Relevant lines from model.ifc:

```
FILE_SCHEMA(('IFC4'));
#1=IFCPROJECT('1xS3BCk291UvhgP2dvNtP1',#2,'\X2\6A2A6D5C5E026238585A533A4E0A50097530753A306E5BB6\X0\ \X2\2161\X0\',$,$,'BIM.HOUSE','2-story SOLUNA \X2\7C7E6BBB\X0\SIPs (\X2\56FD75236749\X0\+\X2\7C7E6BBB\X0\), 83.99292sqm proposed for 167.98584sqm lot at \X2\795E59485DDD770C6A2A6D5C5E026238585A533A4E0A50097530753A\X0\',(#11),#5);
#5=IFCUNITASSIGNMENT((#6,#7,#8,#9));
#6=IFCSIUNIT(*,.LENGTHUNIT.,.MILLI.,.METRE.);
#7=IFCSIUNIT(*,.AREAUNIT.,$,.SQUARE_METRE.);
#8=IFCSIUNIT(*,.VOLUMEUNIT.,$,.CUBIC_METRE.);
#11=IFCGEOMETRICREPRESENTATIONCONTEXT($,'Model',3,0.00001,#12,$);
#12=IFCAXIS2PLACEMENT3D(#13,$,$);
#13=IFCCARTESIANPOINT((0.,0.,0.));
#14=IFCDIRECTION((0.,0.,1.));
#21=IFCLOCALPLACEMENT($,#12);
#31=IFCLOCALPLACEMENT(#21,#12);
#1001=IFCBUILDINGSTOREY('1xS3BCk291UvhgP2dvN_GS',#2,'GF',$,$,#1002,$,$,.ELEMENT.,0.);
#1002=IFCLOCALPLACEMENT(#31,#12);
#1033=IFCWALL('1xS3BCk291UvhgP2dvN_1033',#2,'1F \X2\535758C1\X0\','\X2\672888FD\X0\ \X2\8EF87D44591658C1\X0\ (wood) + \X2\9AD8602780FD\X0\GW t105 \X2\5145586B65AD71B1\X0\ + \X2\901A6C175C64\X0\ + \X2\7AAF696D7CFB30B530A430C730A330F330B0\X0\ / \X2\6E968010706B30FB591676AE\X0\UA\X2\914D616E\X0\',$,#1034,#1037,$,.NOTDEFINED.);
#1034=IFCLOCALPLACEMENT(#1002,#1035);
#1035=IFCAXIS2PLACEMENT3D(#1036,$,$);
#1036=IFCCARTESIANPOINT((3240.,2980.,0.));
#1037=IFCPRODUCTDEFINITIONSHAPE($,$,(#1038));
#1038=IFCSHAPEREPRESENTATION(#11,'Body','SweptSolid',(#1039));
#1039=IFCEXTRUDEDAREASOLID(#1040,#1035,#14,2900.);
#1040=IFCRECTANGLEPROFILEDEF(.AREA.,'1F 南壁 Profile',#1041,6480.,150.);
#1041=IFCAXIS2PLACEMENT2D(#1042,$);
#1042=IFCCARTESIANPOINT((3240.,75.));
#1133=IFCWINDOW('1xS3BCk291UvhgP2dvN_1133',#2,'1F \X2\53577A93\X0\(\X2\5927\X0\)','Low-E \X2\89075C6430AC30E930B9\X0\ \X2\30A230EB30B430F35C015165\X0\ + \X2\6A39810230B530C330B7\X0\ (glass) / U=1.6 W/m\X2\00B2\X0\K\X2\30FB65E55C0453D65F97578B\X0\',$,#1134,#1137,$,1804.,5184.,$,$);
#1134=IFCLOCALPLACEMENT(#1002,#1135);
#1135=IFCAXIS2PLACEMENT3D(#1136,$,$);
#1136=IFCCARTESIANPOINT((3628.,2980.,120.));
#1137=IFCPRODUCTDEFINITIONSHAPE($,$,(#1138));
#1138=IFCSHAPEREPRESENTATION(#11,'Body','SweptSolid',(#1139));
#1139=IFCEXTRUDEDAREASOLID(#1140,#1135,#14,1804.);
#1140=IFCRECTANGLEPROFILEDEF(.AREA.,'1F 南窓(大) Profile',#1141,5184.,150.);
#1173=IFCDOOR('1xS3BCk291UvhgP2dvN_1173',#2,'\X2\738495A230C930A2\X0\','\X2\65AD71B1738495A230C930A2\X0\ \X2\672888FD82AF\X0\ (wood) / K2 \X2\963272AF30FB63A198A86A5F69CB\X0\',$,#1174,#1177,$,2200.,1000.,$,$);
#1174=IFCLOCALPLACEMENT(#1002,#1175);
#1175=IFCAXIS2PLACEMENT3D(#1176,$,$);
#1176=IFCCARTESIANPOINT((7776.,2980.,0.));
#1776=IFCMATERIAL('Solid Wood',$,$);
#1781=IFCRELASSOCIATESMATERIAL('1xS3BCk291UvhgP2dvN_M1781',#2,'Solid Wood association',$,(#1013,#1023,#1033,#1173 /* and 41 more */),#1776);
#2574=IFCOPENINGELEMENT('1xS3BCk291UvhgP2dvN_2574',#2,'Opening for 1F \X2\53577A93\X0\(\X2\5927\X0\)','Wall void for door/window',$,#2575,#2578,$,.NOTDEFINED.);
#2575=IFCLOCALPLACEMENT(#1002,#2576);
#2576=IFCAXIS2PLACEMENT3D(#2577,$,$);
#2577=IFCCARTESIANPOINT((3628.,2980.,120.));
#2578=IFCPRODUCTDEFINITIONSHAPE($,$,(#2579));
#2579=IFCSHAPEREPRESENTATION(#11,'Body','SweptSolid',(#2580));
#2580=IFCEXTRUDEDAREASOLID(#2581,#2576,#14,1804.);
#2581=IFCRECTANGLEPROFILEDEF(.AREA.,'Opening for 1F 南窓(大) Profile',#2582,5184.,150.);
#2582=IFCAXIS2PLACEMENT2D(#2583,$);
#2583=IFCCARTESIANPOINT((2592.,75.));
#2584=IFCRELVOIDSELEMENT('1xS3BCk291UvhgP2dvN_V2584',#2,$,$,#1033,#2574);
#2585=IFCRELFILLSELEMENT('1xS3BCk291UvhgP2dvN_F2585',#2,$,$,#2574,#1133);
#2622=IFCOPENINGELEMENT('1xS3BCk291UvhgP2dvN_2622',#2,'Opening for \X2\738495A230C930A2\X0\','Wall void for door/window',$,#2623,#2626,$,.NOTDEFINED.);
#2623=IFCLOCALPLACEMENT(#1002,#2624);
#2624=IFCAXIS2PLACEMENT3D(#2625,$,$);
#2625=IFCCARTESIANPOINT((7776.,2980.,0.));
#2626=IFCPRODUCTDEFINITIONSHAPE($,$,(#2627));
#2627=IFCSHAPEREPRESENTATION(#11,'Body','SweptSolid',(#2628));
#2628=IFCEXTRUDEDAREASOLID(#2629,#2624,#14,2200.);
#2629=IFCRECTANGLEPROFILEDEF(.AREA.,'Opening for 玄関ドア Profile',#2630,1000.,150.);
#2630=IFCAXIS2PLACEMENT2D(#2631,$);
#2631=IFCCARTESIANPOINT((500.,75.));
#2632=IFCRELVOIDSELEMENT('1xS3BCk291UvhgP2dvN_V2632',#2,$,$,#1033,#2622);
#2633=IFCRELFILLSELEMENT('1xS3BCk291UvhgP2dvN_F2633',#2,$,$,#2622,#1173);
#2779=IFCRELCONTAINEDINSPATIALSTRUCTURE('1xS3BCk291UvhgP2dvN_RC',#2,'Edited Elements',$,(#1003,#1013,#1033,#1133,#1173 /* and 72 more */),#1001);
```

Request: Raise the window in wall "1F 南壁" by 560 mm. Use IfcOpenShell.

```python
import numpy as np
import ifcopenshell
import ifcopenshell.api.geometry
import ifcopenshell.util.placement
import ifcopenshell.util.unit

model = ifcopenshell.open("model.ifc")
unit_scale = ifcopenshell.util.unit.calculate_unit_scale(model)

window = model.by_id(1133)
opening = window.FillsVoids[0].RelatingOpeningElement
dz = 560.0

shift = np.array([0.0, 0.0, dz])
# The window is not placed relative to its opening, so move both.
for product in (opening, window):
    matrix = ifcopenshell.util.placement.get_local_placement(product.ObjectPlacement)
    matrix[:3, 3] += shift
    ifcopenshell.api.geometry.edit_object_placement(model, product=product, matrix=matrix, is_si=False)

print(f"moved by {dz * unit_scale:+.3f} m")

model.write("model_v2.ifc")
```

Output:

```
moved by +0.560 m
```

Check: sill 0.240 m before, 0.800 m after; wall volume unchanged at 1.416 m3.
